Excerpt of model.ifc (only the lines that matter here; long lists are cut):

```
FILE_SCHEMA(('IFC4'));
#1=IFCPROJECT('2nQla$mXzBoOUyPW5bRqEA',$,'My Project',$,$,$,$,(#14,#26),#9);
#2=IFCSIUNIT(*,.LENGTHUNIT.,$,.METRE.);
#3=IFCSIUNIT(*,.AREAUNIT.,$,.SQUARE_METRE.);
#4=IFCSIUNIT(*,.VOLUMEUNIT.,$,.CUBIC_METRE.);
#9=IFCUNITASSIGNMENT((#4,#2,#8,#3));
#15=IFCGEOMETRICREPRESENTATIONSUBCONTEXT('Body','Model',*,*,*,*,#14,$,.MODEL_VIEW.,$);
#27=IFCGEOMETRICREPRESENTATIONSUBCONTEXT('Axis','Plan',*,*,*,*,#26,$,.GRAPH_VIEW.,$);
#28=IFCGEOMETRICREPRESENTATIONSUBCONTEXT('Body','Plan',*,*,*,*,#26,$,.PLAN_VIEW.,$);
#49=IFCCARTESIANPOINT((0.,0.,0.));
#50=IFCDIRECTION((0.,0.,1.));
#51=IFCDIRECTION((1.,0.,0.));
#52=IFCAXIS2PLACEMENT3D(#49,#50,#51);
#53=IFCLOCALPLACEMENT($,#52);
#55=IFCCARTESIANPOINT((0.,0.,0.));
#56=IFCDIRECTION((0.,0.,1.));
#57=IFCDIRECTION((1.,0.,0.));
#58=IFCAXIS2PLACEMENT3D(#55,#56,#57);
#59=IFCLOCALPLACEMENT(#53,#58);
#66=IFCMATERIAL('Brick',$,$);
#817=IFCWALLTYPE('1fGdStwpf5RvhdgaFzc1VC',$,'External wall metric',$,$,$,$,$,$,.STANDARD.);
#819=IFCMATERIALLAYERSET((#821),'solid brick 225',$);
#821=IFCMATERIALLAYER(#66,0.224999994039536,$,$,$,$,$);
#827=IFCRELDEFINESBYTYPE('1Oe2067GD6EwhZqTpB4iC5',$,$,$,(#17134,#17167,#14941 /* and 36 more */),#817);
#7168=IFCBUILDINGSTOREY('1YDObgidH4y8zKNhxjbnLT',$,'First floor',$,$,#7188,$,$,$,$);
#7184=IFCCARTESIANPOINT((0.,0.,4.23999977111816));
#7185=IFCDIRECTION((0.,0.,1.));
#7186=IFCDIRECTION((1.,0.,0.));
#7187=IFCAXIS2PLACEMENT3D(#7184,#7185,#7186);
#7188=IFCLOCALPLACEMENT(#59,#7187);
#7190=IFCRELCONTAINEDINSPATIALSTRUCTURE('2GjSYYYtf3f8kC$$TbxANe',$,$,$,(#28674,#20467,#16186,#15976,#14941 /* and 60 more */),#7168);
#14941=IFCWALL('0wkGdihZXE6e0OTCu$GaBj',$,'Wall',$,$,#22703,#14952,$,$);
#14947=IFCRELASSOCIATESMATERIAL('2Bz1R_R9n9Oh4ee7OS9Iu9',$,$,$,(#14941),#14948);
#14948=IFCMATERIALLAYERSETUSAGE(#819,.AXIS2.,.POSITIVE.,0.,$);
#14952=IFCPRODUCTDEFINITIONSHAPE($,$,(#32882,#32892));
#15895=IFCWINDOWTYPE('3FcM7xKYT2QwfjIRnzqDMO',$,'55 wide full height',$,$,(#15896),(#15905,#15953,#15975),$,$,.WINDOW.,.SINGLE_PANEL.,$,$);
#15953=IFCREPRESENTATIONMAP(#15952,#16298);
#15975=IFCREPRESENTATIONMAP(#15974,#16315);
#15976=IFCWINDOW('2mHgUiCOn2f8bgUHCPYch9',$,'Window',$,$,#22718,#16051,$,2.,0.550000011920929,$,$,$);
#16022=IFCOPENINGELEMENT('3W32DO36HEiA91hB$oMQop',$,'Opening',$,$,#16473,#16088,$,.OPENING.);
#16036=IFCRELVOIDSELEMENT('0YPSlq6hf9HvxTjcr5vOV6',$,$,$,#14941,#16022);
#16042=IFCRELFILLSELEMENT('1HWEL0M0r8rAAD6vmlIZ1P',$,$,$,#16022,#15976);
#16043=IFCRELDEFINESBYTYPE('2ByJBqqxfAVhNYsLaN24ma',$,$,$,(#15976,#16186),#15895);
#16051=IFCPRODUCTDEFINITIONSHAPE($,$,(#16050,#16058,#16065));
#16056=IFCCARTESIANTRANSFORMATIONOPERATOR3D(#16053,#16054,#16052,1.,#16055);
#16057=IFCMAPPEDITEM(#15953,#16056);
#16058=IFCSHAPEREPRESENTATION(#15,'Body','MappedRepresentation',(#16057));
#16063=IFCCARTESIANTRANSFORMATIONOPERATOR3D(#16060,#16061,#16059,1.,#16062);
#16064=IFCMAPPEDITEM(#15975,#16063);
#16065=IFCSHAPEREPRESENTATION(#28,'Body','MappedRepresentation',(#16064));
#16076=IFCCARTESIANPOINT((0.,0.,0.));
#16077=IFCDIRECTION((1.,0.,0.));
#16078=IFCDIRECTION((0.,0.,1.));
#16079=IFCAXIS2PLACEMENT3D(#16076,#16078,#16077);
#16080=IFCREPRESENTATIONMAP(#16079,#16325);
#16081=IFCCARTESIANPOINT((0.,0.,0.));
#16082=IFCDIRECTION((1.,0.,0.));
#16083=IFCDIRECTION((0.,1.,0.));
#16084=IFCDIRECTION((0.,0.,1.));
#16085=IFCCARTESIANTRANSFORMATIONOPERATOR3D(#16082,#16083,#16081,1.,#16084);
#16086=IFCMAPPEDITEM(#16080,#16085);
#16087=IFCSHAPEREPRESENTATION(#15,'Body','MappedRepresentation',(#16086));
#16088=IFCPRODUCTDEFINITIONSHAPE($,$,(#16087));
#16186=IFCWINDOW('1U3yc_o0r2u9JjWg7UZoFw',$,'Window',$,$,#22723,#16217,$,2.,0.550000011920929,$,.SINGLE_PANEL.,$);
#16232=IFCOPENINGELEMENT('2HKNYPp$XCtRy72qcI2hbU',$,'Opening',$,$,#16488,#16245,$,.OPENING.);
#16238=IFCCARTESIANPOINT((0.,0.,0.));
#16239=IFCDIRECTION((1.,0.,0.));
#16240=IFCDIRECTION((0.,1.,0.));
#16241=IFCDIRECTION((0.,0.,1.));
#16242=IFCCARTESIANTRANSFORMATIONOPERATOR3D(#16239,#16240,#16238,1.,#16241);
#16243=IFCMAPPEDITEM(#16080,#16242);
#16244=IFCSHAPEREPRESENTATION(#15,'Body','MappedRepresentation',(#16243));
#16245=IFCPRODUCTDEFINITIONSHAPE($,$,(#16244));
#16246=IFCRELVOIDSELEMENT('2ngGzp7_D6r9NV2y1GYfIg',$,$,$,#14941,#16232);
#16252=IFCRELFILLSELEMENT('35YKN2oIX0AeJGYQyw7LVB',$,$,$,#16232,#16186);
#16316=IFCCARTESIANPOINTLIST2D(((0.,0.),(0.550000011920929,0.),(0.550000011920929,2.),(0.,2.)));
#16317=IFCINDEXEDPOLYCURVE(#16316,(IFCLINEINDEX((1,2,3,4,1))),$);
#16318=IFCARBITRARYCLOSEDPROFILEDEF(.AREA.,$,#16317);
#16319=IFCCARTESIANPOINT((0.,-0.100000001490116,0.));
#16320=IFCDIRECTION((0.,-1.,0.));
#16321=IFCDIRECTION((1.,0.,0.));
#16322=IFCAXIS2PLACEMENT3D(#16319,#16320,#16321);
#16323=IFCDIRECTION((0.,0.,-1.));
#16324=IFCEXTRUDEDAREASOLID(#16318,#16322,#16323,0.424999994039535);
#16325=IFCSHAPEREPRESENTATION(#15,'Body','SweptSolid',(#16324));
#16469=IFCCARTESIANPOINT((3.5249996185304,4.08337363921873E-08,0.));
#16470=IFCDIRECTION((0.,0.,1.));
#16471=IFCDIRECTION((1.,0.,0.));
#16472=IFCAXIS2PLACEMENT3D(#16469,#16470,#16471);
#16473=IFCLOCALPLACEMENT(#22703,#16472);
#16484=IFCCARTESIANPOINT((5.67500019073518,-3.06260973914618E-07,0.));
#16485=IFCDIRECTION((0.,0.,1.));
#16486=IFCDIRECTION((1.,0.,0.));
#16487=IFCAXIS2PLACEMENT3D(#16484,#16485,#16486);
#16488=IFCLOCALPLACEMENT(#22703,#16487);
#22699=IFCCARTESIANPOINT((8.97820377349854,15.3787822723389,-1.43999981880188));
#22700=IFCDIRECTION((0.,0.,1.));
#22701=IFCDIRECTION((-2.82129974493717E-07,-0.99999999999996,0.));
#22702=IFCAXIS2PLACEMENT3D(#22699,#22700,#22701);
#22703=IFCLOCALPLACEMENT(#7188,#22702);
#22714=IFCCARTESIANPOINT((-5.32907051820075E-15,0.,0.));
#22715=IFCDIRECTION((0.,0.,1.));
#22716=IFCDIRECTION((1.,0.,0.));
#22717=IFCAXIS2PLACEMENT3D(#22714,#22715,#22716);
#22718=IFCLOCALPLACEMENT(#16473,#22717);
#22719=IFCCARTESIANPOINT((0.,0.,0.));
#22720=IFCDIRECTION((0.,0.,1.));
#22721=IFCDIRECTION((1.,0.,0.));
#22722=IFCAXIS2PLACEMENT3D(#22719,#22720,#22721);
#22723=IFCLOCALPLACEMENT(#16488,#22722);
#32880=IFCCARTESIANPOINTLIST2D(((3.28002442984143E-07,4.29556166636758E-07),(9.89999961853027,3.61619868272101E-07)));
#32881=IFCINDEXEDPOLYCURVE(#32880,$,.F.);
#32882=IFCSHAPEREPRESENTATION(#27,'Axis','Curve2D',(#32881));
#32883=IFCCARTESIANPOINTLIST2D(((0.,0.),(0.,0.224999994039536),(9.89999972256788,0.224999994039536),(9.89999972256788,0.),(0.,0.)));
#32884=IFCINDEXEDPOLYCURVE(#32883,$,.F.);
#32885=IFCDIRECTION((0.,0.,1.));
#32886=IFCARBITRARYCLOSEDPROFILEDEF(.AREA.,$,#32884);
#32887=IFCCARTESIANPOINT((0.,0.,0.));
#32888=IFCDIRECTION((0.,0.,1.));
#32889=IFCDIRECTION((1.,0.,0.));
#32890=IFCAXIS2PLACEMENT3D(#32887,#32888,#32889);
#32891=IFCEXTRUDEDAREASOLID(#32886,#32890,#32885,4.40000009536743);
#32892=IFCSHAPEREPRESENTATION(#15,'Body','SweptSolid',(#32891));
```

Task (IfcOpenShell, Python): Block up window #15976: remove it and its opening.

```python
import ifcopenshell
import ifcopenshell.api.feature
import ifcopenshell.api.root
import ifcopenshell.geom
import ifcopenshell.util.shape

model = ifcopenshell.open("model.ifc")
settings = ifcopenshell.geom.settings()


def volume(element):
    """Net volume in cubic metres, openings subtracted."""
    shape = ifcopenshell.geom.create_shape(settings, element)
    return ifcopenshell.util.shape.get_volume(shape.geometry)


window = model.by_guid("2mHgUiCOn2f8bgUHCPYch9")
opening = window.FillsVoids[0].RelatingOpeningElement
wall = opening.VoidsElements[0].RelatingBuildingElement
before = volume(wall)

ifcopenshell.api.root.remove_product(model, product=window)
ifcopenshell.api.feature.remove_feature(model, feature=opening)

after = volume(wall)

print(f"wall volume {before:.3f} -> {after:.3f} m3")

model.write("model-out.ifc")
```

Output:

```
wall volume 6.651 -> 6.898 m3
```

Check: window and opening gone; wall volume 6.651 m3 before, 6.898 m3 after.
